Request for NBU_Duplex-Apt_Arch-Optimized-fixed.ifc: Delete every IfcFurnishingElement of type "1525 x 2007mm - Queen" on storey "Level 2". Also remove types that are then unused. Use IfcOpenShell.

First a look at what the model holds.

```python
import ifcopenshell
import ifcopenshell.util.element

model = ifcopenshell.open("NBU_Duplex-Apt_Arch-Optimized-fixed.ifc")
print(model.schema)
storey = next(s for s in model.by_type("IfcBuildingStorey") if s.Name == "Level 2")
furniture = [e for e in ifcopenshell.util.element.get_decomposition(storey) if e.is_a("IfcFurnishingElement")]
seen = {}
for e in furniture:
    element_type = ifcopenshell.util.element.get_type(e)
    name = element_type.Name if element_type not in (None, e) else None
    seen[name] = seen.get(name, 0) + 1
for name, count in sorted(seen.items(), key=str):
    print(count, "x", name)
```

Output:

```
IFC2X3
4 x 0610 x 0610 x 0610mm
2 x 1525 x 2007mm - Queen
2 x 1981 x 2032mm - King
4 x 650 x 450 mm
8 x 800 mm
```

```python
import ifcopenshell
import ifcopenshell.api.root
import ifcopenshell.util.element

model = ifcopenshell.open("NBU_Duplex-Apt_Arch-Optimized-fixed.ifc")

storey = next(s for s in model.by_type("IfcBuildingStorey") if s.Name == "Level 2")
furniture = [e for e in ifcopenshell.util.element.get_decomposition(storey) if e.is_a("IfcFurnishingElement")]
targets = [e for e in furniture if (t := ifcopenshell.util.element.get_type(e)) not in (None, e) and t.Name == "1525 x 2007mm - Queen"]
types = {ifcopenshell.util.element.get_type(e) for e in targets} - {None, *targets}

for e in targets:
    ifcopenshell.api.root.remove_product(model, product=e)
print(len(targets), "removed")

unused = [t for t in types if not ifcopenshell.util.element.get_types(t)]
for t in unused:
    ifcopenshell.api.root.remove_product(model, product=t)
print(len(unused), "unused types removed")

model.write("NBU_Duplex-Apt_Arch-Optimized-fixed_updated.ifc")
```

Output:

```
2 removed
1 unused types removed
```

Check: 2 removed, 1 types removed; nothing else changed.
